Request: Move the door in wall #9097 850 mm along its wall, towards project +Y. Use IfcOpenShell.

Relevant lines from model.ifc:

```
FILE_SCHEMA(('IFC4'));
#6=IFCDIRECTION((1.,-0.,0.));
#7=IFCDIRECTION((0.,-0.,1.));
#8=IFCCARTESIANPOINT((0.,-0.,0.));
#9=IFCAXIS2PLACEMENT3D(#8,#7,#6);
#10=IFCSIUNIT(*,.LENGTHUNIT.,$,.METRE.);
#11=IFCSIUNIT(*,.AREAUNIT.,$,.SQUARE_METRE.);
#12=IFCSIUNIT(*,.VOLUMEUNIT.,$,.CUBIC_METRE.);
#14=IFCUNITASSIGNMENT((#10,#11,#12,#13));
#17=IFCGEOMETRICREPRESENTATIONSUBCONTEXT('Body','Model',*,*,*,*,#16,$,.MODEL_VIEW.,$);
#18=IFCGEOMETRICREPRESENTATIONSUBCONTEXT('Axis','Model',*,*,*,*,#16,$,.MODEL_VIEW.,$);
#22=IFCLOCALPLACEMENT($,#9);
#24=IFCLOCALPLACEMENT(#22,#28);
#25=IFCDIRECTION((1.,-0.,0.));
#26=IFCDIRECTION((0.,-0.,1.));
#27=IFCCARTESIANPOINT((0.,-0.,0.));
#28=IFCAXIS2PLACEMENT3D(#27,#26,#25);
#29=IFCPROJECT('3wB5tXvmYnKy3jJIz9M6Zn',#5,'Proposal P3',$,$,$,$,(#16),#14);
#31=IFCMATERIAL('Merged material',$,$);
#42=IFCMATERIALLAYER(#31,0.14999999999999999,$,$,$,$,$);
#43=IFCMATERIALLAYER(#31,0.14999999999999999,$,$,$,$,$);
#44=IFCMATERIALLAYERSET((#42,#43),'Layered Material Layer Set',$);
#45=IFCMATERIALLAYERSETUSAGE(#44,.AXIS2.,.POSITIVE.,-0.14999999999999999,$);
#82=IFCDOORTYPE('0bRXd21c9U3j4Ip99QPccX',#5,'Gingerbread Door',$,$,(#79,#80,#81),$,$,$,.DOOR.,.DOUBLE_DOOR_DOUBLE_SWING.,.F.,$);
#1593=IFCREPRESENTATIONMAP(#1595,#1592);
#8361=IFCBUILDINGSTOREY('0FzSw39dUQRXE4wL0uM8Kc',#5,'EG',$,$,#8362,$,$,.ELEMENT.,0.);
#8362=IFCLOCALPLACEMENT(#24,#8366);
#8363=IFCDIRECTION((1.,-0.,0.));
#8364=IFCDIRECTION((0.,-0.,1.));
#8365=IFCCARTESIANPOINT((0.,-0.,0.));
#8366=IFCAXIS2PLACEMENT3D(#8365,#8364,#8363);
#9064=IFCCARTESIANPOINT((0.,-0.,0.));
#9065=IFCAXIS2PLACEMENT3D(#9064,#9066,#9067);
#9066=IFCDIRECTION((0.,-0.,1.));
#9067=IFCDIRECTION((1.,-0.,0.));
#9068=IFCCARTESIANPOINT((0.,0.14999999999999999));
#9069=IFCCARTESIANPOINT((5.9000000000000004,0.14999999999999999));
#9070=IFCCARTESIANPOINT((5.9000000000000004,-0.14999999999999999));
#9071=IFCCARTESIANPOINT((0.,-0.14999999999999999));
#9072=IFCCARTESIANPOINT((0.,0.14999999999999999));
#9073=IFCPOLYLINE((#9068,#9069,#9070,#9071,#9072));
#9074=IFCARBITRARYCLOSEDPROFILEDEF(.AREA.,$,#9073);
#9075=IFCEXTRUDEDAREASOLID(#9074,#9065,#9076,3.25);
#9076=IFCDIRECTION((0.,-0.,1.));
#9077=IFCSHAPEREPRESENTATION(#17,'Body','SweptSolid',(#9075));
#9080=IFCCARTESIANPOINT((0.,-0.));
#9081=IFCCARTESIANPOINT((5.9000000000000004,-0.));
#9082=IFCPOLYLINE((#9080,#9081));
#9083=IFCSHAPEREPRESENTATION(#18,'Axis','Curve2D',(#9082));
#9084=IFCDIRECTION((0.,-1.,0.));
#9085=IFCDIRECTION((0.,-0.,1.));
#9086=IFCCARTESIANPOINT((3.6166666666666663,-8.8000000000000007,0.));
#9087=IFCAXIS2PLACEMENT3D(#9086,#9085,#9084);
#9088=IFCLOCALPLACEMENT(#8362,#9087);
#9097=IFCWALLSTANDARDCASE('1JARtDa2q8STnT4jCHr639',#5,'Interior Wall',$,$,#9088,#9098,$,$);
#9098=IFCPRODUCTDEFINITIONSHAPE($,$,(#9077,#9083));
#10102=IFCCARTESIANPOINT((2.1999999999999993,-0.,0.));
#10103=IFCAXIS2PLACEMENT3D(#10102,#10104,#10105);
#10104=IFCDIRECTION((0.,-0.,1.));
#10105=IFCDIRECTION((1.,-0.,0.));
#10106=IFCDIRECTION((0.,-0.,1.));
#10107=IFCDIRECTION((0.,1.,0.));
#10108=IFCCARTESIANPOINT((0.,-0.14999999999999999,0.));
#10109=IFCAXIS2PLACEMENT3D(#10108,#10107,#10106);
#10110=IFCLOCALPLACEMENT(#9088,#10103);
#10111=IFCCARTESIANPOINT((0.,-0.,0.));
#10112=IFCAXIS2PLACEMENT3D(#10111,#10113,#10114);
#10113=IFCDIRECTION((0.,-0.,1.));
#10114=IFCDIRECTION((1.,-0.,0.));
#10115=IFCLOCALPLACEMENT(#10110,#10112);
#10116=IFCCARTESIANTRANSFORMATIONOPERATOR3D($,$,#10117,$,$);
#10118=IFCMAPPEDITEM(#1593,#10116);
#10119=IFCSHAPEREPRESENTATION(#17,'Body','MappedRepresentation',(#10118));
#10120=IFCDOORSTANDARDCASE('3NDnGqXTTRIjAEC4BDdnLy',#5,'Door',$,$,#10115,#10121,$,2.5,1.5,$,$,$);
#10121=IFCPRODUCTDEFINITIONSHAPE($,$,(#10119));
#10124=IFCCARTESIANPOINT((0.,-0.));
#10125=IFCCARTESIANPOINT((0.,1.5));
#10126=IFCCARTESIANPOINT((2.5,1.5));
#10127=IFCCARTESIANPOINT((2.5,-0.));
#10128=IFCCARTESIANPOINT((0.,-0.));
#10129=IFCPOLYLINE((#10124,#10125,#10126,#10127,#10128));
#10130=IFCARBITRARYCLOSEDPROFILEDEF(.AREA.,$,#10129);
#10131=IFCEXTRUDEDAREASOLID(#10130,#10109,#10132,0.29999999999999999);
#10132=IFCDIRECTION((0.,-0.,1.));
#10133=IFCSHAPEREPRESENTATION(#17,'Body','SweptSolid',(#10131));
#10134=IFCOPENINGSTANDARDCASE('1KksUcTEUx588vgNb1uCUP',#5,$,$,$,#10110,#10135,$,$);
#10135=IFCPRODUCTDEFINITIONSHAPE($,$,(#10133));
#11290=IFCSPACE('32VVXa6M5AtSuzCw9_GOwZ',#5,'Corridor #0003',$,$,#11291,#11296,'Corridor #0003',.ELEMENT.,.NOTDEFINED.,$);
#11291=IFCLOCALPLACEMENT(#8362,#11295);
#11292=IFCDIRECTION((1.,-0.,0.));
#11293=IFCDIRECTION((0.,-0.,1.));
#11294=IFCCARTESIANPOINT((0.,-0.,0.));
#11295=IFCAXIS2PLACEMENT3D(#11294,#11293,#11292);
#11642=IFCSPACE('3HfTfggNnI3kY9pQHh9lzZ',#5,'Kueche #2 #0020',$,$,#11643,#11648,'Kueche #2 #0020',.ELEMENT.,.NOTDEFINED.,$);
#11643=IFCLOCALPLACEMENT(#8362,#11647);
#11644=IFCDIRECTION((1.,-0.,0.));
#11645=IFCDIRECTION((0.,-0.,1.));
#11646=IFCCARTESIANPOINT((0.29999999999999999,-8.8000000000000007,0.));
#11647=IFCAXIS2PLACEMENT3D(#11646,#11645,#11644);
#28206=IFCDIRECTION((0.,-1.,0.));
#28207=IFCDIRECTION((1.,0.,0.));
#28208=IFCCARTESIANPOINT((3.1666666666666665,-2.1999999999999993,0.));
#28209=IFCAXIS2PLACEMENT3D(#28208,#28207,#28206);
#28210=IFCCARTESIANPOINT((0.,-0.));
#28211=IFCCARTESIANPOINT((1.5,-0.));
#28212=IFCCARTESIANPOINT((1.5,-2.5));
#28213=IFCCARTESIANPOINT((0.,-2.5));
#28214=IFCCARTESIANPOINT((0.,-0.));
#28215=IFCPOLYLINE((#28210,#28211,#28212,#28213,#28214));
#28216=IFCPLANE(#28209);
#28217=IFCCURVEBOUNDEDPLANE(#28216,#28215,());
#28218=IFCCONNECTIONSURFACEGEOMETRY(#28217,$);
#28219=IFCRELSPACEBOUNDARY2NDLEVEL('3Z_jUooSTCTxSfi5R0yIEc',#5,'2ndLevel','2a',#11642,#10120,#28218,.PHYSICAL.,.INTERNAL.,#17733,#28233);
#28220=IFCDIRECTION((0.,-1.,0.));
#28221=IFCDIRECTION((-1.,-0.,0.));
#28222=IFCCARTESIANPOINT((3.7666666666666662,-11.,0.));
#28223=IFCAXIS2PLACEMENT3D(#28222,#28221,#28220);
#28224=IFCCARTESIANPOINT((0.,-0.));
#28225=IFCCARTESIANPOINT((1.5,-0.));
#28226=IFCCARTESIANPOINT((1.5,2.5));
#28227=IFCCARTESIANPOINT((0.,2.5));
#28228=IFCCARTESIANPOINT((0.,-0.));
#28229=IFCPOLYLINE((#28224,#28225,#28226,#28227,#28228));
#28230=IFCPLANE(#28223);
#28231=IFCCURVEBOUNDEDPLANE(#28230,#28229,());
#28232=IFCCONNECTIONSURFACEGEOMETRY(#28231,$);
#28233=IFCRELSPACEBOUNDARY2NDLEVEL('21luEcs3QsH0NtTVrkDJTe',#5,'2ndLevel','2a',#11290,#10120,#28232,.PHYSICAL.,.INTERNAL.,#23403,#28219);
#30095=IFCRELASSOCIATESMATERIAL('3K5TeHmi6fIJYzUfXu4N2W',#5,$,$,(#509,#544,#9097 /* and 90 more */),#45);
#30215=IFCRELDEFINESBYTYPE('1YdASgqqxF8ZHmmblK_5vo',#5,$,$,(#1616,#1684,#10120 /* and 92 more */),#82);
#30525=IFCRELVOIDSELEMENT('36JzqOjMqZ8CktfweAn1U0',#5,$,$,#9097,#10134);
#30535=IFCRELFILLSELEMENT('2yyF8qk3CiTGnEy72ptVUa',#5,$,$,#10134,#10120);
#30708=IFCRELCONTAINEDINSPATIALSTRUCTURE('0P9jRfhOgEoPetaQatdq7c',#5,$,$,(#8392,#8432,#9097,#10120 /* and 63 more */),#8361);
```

```python
import numpy as np
import ifcopenshell
import ifcopenshell.api.geometry
import ifcopenshell.util.placement

model = ifcopenshell.open("model.ifc")

door = model.by_guid("3NDnGqXTTRIjAEC4BDdnLy")
opening = door.FillsVoids[0].RelatingOpeningElement
wall = opening.VoidsElements[0].RelatingBuildingElement

wall_matrix = ifcopenshell.util.placement.get_local_placement(wall.ObjectPlacement)
shift = wall_matrix[:3, 0] * -0.85
before = ifcopenshell.util.placement.get_local_placement(door.ObjectPlacement)[:3, 3].copy()

# The door is placed relative to its opening, so it follows when the opening moves.
matrix = ifcopenshell.util.placement.get_local_placement(opening.ObjectPlacement)
matrix[:3, 3] += shift
ifcopenshell.api.geometry.edit_object_placement(
    model, product=opening, matrix=matrix, is_si=False, should_transform_children=True
)

# Space boundary surfaces are stored in each space's coordinates; move them too.
for rel in door.ProvidesBoundaries:
    if not rel.ConnectionGeometry:
        continue
    surface = rel.ConnectionGeometry.SurfaceOnRelatingElement.BasisSurface
    space_matrix = ifcopenshell.util.placement.get_local_placement(rel.RelatingSpace.ObjectPlacement)
    point = np.array(surface.Position.Location.Coordinates) + space_matrix[:3, :3].T @ shift
    surface.Position = model.createIfcAxis2Placement3D(
        model.createIfcCartesianPoint(point.tolist()), surface.Position.Axis, surface.Position.RefDirection
    )

after = ifcopenshell.util.placement.get_local_placement(door.ObjectPlacement)[:3, 3]
print("door moved by", (after - before).round(3) + 0.0)

model.write("model_v2.ifc")
```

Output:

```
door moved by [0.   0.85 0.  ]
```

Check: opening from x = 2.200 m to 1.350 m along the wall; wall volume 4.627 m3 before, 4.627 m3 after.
